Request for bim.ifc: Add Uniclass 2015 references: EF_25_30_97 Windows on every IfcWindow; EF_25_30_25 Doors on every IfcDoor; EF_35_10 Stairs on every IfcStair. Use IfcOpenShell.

First a look at what the model holds.

```python
import ifcopenshell

model = ifcopenshell.open("bim.ifc")
print(model.schema)
print("classifications:", [c.Name for c in model.by_type("IfcClassification")])
for ifc_class in ("IfcDoor", "IfcRoof", "IfcStair", "IfcWall", "IfcWindow"):
    print(ifc_class, len(model.by_type(ifc_class)))
```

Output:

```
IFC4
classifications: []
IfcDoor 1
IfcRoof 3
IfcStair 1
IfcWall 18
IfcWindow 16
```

```python
import ifcopenshell
import ifcopenshell.api.classification

model = ifcopenshell.open("bim.ifc")

system = ifcopenshell.api.classification.add_classification(model, classification="Uniclass 2015")

codes = {
    "IfcWindow": ("EF_25_30_97", "Windows"),
    "IfcDoor": ("EF_25_30_25", "Doors"),
    "IfcStair": ("EF_35_10", "Stairs"),
}
for ifc_class, (code, name) in codes.items():
    products = model.by_type(ifc_class)
    ifcopenshell.api.classification.add_reference(
        model, products=products, classification=system, identification=code, name=name
    )
    print(code, len(products))

model.write("bim-out.ifc")
```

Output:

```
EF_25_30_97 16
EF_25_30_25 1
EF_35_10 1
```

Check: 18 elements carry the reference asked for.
